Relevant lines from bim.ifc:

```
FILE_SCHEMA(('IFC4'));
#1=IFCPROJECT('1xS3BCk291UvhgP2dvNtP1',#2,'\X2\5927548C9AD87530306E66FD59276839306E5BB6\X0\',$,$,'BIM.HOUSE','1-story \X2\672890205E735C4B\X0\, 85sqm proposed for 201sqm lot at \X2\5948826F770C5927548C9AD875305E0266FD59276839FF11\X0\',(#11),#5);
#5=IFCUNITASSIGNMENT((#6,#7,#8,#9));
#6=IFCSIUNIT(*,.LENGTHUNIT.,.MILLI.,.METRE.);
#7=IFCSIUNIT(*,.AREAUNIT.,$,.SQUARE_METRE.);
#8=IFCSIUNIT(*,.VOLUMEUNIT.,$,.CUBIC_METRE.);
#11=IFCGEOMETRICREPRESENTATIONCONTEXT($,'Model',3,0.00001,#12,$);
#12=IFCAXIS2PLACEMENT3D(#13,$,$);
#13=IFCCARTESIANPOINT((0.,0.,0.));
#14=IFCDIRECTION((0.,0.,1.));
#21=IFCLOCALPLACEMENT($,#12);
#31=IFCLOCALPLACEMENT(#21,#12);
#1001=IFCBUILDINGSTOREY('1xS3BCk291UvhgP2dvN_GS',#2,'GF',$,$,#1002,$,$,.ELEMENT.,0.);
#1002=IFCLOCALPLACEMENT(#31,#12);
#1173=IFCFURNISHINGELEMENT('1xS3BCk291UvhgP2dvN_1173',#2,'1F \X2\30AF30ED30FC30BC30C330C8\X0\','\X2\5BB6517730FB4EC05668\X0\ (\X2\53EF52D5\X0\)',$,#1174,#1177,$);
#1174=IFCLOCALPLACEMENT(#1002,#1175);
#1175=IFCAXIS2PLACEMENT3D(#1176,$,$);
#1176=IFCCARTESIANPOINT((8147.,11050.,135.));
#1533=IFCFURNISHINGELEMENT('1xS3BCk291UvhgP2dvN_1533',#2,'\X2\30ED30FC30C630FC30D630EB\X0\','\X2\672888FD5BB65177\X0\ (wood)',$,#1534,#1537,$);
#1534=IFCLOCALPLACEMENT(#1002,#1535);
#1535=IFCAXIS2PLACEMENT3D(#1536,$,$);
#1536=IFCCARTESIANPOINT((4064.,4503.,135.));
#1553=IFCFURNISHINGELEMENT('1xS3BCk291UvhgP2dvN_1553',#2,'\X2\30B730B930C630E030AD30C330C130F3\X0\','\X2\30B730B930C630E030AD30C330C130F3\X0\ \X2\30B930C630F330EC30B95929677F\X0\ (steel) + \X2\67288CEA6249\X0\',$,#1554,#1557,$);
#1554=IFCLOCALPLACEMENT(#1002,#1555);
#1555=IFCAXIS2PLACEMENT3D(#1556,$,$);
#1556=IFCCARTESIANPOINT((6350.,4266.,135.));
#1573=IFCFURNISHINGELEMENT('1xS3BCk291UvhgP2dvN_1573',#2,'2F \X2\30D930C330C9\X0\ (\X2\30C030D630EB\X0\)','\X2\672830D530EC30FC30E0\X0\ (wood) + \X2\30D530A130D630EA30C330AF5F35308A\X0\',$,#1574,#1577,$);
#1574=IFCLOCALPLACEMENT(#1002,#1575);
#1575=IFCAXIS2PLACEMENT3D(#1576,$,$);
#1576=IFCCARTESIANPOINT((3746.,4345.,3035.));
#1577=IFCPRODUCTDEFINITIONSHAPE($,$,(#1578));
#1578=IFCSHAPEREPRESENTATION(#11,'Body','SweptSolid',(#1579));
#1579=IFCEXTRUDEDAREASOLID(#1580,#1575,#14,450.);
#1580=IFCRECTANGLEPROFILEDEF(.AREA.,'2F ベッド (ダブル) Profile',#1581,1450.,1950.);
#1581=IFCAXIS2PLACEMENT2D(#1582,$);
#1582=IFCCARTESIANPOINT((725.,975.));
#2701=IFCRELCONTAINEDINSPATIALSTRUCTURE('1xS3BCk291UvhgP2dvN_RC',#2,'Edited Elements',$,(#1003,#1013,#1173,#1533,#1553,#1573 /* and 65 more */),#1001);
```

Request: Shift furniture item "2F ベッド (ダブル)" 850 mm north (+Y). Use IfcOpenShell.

```python
import ifcopenshell
import ifcopenshell.api.geometry
import ifcopenshell.util.placement

model = ifcopenshell.open("bim.ifc")

item = model.by_guid("1xS3BCk291UvhgP2dvN_1573")
matrix = ifcopenshell.util.placement.get_local_placement(item.ObjectPlacement)
matrix[1, 3] += 850.0
ifcopenshell.api.geometry.edit_object_placement(model, product=item, matrix=matrix, is_si=False)

print(ifcopenshell.util.placement.get_local_placement(item.ObjectPlacement).round(3) + 0.0)

model.write("bim_rev.ifc")
```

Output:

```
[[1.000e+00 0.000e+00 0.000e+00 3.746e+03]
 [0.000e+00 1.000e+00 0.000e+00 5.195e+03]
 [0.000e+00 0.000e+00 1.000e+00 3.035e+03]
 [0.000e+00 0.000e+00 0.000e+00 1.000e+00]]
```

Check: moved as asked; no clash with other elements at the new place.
